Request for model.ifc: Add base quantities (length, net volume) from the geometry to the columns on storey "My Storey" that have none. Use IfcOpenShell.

First a look at what the model holds.

```python
import ifcopenshell
import ifcopenshell.util.element
import ifcopenshell.util.unit

model = ifcopenshell.open("model.ifc")
print(model.schema)
for unit_type in ("LENGTHUNIT", "AREAUNIT", "VOLUMEUNIT"):
    print(unit_type, ifcopenshell.util.unit.calculate_unit_scale(model, unit_type))
storey = next(s for s in model.by_type("IfcBuildingStorey") if s.Name == "My Storey")
columns = [e for e in ifcopenshell.util.element.get_decomposition(storey) if e.is_a("IfcColumn")]
for e in sorted(columns, key=lambda e: e.id()):
    print(e.id(), e.is_a(), e.Name, list(ifcopenshell.util.element.get_psets(e, qtos_only=True)), sep=" | ")
```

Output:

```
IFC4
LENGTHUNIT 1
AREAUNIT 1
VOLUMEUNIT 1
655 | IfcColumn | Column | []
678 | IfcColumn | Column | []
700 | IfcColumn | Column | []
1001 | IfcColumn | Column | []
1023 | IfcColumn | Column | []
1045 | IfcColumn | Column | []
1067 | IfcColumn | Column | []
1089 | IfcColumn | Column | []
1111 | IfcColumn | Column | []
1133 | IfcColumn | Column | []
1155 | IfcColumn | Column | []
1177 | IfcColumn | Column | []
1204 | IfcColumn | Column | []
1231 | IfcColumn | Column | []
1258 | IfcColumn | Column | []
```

```python
import ifcopenshell
import ifcopenshell.api.pset
import ifcopenshell.geom
import ifcopenshell.util.element
import ifcopenshell.util.shape
import ifcopenshell.util.unit

model = ifcopenshell.open("model.ifc")
unit_scale = ifcopenshell.util.unit.calculate_unit_scale(model)
volume_scale = ifcopenshell.util.unit.calculate_unit_scale(model, "VOLUMEUNIT")
settings = ifcopenshell.geom.settings()

storey = next(s for s in model.by_type("IfcBuildingStorey") if s.Name == "My Storey")
columns = [e for e in ifcopenshell.util.element.get_decomposition(storey) if e.is_a("IfcColumn")]

for e in sorted(columns, key=lambda e: e.id()):
    if ifcopenshell.util.element.get_psets(e, qtos_only=True, should_inherit=False):
        continue
    # Geometry comes back in metres, in the element's own axes.
    shape = ifcopenshell.geom.create_shape(settings, e)
    values = {
        "Length": ifcopenshell.util.shape.get_z(shape.geometry) / unit_scale,
        "NetVolume": ifcopenshell.util.shape.get_volume(shape.geometry) / volume_scale,
    }
    qto = ifcopenshell.api.pset.add_qto(model, product=e, name="Qto_ColumnBaseQuantities")
    ifcopenshell.api.pset.edit_qto(model, qto=qto, properties=values)
    print(e.id(), {k: round(v, 3) for k, v in values.items()})

model.write("model_edited.ifc")
```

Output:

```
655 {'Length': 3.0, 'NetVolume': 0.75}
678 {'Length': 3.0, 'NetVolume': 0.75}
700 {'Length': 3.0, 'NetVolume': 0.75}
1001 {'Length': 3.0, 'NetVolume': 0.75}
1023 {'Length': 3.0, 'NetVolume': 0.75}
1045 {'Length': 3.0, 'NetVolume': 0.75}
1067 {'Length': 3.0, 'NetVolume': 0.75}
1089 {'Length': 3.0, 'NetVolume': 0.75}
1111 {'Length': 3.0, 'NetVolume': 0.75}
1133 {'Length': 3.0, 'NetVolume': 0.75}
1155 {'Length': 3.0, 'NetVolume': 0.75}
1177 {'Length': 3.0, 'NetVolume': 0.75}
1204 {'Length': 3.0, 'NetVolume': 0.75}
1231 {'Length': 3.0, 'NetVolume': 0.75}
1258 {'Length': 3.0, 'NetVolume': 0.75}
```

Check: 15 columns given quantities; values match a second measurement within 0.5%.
